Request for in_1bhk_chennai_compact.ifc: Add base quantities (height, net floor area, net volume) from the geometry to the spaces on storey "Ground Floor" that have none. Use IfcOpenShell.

First a look at what the model holds.

```python
import ifcopenshell
import ifcopenshell.util.element
import ifcopenshell.util.unit

model = ifcopenshell.open("in_1bhk_chennai_compact.ifc")
print(model.schema)
for unit_type in ("LENGTHUNIT", "AREAUNIT", "VOLUMEUNIT"):
    print(unit_type, ifcopenshell.util.unit.calculate_unit_scale(model, unit_type))
storey = next(s for s in model.by_type("IfcBuildingStorey") if s.Name == "Ground Floor")
spaces = [e for e in ifcopenshell.util.element.get_decomposition(storey) if e.is_a("IfcSpace")]
for e in sorted(spaces, key=lambda e: e.id()):
    print(e.id(), e.is_a(), e.Name, list(ifcopenshell.util.element.get_psets(e, qtos_only=True)), sep=" | ")
```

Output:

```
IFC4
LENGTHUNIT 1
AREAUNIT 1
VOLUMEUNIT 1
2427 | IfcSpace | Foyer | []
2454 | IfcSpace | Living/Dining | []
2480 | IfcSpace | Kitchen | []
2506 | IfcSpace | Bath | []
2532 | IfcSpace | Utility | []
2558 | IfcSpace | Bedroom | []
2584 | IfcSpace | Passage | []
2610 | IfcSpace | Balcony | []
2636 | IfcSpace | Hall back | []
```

```python
import ifcopenshell
import ifcopenshell.api.pset
import ifcopenshell.geom
import ifcopenshell.util.element
import ifcopenshell.util.shape
import ifcopenshell.util.unit

model = ifcopenshell.open("in_1bhk_chennai_compact.ifc")
unit_scale = ifcopenshell.util.unit.calculate_unit_scale(model)
area_scale = ifcopenshell.util.unit.calculate_unit_scale(model, "AREAUNIT")
volume_scale = ifcopenshell.util.unit.calculate_unit_scale(model, "VOLUMEUNIT")
settings = ifcopenshell.geom.settings()

storey = next(s for s in model.by_type("IfcBuildingStorey") if s.Name == "Ground Floor")
spaces = [e for e in ifcopenshell.util.element.get_decomposition(storey) if e.is_a("IfcSpace")]

for e in sorted(spaces, key=lambda e: e.id()):
    if ifcopenshell.util.element.get_psets(e, qtos_only=True, should_inherit=False):
        continue
    # Geometry comes back in metres, in the element's own axes.
    shape = ifcopenshell.geom.create_shape(settings, e)
    values = {
        "Height": ifcopenshell.util.shape.get_z(shape.geometry) / unit_scale,
        "NetFloorArea": ifcopenshell.util.shape.get_footprint_area(shape.geometry) / area_scale,
        "NetVolume": ifcopenshell.util.shape.get_volume(shape.geometry) / volume_scale,
    }
    qto = ifcopenshell.api.pset.add_qto(model, product=e, name="Qto_SpaceBaseQuantities")
    ifcopenshell.api.pset.edit_qto(model, qto=qto, properties=values)
    print(e.id(), {k: round(v, 3) for k, v in values.items()})

model.write("in_1bhk_chennai_compact_v2.ifc")
```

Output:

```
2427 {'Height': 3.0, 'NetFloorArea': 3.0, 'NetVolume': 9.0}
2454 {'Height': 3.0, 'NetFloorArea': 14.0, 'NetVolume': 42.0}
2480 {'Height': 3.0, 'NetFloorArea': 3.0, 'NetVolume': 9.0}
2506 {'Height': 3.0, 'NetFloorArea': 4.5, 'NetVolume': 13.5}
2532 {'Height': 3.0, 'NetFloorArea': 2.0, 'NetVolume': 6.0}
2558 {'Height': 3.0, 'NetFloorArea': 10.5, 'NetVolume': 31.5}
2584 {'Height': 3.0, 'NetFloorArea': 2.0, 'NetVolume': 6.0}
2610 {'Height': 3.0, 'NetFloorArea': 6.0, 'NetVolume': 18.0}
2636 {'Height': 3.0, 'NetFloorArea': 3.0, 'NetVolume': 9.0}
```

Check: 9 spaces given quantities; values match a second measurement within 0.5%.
